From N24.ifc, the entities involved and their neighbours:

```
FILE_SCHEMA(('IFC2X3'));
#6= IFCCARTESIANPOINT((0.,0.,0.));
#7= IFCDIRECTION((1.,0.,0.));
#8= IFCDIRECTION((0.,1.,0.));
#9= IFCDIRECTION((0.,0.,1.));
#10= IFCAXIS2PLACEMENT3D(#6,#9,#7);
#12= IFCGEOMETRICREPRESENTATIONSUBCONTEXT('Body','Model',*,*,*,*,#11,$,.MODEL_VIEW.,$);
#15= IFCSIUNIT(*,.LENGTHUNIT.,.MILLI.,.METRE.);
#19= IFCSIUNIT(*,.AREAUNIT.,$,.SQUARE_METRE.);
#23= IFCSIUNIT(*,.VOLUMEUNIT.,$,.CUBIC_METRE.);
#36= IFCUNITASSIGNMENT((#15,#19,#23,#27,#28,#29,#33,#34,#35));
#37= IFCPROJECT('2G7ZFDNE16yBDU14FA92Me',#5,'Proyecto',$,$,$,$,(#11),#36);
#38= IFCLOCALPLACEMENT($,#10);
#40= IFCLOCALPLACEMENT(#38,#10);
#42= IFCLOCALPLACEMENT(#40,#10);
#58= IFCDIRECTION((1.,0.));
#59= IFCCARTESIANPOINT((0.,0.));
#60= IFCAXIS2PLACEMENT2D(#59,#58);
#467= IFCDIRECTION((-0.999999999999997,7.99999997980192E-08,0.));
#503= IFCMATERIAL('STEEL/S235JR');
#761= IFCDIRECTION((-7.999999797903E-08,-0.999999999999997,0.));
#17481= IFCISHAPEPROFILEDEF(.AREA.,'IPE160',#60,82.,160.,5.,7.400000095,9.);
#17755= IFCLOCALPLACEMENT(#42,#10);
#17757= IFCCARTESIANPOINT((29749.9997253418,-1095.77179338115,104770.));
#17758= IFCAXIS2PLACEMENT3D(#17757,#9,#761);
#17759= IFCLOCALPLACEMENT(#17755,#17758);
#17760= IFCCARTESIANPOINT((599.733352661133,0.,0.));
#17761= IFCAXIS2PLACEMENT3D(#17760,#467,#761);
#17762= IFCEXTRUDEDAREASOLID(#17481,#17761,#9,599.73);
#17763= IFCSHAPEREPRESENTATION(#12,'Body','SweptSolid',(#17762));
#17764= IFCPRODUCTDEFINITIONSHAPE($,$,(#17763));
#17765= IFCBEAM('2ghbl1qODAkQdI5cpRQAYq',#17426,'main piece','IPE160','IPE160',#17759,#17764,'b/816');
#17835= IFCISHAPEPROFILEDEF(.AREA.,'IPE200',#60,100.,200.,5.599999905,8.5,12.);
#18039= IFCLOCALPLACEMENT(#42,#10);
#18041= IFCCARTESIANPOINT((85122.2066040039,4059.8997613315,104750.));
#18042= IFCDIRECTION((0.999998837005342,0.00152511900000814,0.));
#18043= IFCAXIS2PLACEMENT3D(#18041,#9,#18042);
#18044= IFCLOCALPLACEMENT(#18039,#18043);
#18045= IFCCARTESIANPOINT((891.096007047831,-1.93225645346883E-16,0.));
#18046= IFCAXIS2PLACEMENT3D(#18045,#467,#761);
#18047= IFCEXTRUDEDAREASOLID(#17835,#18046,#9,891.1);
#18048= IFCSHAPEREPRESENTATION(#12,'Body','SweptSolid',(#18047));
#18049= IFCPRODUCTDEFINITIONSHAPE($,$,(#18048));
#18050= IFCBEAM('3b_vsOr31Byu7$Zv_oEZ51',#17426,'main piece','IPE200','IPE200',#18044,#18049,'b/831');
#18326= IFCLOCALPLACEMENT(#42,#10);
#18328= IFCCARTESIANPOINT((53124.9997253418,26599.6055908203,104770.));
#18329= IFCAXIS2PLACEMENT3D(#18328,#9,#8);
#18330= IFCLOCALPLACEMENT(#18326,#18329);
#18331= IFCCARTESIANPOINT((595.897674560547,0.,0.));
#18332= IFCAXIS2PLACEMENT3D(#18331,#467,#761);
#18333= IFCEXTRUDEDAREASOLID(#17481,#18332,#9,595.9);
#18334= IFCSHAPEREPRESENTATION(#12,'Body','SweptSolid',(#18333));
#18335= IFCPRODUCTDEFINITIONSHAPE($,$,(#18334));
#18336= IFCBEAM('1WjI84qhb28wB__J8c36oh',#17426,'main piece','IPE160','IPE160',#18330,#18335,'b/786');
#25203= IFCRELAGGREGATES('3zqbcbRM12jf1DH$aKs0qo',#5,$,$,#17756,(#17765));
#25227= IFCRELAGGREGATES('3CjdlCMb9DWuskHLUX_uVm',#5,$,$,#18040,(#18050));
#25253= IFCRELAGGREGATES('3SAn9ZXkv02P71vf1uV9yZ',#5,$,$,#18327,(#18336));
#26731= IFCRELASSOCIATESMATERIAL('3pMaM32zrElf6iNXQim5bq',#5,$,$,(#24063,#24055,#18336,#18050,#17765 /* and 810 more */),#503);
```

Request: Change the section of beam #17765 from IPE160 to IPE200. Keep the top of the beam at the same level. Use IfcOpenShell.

```python
import ifcopenshell
import ifcopenshell.util.element
import ifcopenshell.util.representation

model = ifcopenshell.open("N24.ifc")

member = model.by_guid("2ghbl1qODAkQdI5cpRQAYq")
source = next(p for p in model.by_type("IfcIShapeProfileDef") if p.ProfileName == "IPE200")

body = ifcopenshell.util.representation.get_representation(member, "Model", "Body")
solid = body.Items[0]
old_profile = solid.SweptArea

# Copy the section's sizes but keep this member's own profile position.
profile = ifcopenshell.util.element.copy(model, source)
# Profiles are centred, so shift by half the change in depth to hold the top.
shift = (old_profile.OverallDepth - profile.OverallDepth) / 2
x, y = old_profile.Position.Location.Coordinates
up = (0.0, 1.0)  # upwards, in the solid's own plane
location = model.createIfcCartesianPoint((x + up[0] * shift, y + up[1] * shift))
profile.Position = model.createIfcAxis2Placement2D(location, old_profile.Position.RefDirection)
solid.SweptArea = profile
if not model.get_total_inverses(old_profile):
    ifcopenshell.util.element.remove_deep2(model, old_profile)
member.Description = member.Description.replace("IPE160", "IPE200")
member.ObjectType = member.ObjectType.replace("IPE160", "IPE200")

print(solid.SweptArea)

model.write("N24_updated.ifc")
```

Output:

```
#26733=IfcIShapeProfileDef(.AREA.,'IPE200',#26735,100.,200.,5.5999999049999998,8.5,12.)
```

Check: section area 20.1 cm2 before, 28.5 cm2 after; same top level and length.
